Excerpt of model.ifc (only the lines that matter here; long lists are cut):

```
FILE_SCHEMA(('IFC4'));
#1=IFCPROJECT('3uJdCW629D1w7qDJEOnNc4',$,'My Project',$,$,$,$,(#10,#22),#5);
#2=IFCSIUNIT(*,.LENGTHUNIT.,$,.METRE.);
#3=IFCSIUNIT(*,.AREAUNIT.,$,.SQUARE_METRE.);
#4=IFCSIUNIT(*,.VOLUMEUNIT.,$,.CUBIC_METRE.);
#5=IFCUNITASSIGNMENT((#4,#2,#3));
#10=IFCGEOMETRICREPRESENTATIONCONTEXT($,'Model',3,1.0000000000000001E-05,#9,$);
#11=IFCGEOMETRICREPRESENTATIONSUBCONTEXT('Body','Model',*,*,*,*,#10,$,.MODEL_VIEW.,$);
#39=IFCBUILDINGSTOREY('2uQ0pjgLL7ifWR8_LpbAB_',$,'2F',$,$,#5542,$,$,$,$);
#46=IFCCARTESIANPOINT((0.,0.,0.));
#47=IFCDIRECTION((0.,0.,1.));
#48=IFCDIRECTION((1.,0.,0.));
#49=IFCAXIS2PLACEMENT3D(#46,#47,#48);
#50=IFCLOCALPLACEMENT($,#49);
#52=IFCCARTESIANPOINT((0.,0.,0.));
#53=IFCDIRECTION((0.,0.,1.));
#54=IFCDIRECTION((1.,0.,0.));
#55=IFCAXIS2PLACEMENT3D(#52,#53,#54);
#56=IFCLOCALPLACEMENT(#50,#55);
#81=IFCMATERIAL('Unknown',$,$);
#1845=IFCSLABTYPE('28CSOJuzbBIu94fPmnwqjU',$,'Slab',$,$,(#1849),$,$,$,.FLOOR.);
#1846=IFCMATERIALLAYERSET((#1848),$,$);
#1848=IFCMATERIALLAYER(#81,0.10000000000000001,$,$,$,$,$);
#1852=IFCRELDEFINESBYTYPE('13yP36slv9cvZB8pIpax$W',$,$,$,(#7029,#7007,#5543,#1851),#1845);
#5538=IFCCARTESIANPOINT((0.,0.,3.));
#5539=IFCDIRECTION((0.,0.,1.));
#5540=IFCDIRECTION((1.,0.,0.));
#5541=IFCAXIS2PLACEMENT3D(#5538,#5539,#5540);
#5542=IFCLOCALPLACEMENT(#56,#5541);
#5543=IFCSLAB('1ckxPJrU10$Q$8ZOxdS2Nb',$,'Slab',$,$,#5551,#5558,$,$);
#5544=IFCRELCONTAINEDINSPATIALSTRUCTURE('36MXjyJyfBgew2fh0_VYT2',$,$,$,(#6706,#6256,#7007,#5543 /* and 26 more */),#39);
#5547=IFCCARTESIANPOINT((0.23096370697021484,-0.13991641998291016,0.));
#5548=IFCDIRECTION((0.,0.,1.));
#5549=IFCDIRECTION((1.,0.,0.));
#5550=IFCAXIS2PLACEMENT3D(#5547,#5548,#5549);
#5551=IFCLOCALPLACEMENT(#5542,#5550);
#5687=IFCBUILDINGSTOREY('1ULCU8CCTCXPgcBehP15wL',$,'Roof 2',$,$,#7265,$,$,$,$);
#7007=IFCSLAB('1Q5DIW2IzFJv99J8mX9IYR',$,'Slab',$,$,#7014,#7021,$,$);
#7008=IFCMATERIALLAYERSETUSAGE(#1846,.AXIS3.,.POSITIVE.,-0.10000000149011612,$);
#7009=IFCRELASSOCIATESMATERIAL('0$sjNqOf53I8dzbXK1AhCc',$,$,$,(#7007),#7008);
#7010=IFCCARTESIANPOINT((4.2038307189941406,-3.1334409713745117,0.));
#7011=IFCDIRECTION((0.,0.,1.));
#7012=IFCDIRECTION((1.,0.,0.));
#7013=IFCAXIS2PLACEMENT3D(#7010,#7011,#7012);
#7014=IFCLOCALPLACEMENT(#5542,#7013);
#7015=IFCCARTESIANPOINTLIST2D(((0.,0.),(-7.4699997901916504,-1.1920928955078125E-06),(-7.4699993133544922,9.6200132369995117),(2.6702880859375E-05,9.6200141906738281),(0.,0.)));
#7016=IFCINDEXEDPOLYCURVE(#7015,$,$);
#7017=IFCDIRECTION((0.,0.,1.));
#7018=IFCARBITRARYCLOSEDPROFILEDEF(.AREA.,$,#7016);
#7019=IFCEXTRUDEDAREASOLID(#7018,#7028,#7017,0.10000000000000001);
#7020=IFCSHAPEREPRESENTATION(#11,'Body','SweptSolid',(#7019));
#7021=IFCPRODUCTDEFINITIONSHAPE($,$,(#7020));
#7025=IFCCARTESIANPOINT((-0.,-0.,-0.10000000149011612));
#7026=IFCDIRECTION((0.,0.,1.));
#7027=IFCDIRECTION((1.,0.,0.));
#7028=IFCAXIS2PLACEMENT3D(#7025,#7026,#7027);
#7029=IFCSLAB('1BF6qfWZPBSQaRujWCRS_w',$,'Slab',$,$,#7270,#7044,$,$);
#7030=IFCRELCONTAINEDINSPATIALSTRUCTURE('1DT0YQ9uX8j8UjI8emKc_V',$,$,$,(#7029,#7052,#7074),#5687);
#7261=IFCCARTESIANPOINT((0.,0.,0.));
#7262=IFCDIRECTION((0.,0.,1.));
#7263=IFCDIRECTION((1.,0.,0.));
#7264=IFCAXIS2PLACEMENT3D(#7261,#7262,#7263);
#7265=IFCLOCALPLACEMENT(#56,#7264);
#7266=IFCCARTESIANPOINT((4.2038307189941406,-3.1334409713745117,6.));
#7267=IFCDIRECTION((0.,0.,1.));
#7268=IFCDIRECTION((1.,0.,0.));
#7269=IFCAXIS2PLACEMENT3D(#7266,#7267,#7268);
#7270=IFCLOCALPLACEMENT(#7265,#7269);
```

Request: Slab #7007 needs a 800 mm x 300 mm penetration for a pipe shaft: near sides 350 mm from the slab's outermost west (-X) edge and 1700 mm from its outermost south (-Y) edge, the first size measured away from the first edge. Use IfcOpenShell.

```python
import numpy as np
import ifcopenshell
import ifcopenshell.api.feature
import ifcopenshell.api.geometry
import ifcopenshell.api.root
import ifcopenshell.geom
import ifcopenshell.util.placement
import ifcopenshell.util.representation
import ifcopenshell.util.shape
import ifcopenshell.util.unit

model = ifcopenshell.open("model.ifc")
unit_scale = ifcopenshell.util.unit.calculate_unit_scale(model)
settings = ifcopenshell.geom.settings()


def volume(element):
    """Net volume in cubic metres, openings subtracted."""
    shape = ifcopenshell.geom.create_shape(settings, element)
    return ifcopenshell.util.shape.get_volume(shape.geometry)


slab = model.by_guid("1Q5DIW2IzFJv99J8mX9IYR")
before = volume(slab)

# Extent in the slab's own axes, in metres. The edges named are its -X and -Y sides.
slab_shape = ifcopenshell.geom.create_shape(settings, slab)
vertices = ifcopenshell.util.shape.get_vertices(slab_shape.geometry)
x_min, y_min, bottom = vertices.min(axis=0)
top = vertices[:, 2].max()

opening = ifcopenshell.api.root.create_entity(model, ifc_class="IfcOpeningElement", name="Pipe shaft opening", predefined_type="OPENING")
context = ifcopenshell.util.representation.get_context(model, "Model", "Body", "MODEL_VIEW")
width, depth = 0.8, 0.3
outline = [(0.0, 0.0), (width, 0.0), (width, depth), (0.0, depth), (0.0, 0.0)]
# Overshoot both faces by 50 mm so the cut is clean.
shape = ifcopenshell.api.geometry.add_slab_representation(
    model, context=context, depth=top - bottom + 0.1, polyline=outline
)
ifcopenshell.api.geometry.assign_representation(model, product=opening, representation=shape)

matrix = ifcopenshell.util.placement.get_local_placement(slab.ObjectPlacement)
matrix[:, 3] = matrix @ np.append(np.array([x_min + 0.35, y_min + 1.7, bottom - 0.05]) / unit_scale, 1.0)
ifcopenshell.api.geometry.edit_object_placement(model, product=opening, matrix=matrix, is_si=False)
ifcopenshell.api.feature.add_feature(model, feature=opening, element=slab)

after = volume(slab)

print(f"slab volume {before:.3f} -> {after:.3f} m3")

model.write("model-out.ifc")
```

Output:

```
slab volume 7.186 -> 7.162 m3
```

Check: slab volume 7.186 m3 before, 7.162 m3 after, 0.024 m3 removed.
